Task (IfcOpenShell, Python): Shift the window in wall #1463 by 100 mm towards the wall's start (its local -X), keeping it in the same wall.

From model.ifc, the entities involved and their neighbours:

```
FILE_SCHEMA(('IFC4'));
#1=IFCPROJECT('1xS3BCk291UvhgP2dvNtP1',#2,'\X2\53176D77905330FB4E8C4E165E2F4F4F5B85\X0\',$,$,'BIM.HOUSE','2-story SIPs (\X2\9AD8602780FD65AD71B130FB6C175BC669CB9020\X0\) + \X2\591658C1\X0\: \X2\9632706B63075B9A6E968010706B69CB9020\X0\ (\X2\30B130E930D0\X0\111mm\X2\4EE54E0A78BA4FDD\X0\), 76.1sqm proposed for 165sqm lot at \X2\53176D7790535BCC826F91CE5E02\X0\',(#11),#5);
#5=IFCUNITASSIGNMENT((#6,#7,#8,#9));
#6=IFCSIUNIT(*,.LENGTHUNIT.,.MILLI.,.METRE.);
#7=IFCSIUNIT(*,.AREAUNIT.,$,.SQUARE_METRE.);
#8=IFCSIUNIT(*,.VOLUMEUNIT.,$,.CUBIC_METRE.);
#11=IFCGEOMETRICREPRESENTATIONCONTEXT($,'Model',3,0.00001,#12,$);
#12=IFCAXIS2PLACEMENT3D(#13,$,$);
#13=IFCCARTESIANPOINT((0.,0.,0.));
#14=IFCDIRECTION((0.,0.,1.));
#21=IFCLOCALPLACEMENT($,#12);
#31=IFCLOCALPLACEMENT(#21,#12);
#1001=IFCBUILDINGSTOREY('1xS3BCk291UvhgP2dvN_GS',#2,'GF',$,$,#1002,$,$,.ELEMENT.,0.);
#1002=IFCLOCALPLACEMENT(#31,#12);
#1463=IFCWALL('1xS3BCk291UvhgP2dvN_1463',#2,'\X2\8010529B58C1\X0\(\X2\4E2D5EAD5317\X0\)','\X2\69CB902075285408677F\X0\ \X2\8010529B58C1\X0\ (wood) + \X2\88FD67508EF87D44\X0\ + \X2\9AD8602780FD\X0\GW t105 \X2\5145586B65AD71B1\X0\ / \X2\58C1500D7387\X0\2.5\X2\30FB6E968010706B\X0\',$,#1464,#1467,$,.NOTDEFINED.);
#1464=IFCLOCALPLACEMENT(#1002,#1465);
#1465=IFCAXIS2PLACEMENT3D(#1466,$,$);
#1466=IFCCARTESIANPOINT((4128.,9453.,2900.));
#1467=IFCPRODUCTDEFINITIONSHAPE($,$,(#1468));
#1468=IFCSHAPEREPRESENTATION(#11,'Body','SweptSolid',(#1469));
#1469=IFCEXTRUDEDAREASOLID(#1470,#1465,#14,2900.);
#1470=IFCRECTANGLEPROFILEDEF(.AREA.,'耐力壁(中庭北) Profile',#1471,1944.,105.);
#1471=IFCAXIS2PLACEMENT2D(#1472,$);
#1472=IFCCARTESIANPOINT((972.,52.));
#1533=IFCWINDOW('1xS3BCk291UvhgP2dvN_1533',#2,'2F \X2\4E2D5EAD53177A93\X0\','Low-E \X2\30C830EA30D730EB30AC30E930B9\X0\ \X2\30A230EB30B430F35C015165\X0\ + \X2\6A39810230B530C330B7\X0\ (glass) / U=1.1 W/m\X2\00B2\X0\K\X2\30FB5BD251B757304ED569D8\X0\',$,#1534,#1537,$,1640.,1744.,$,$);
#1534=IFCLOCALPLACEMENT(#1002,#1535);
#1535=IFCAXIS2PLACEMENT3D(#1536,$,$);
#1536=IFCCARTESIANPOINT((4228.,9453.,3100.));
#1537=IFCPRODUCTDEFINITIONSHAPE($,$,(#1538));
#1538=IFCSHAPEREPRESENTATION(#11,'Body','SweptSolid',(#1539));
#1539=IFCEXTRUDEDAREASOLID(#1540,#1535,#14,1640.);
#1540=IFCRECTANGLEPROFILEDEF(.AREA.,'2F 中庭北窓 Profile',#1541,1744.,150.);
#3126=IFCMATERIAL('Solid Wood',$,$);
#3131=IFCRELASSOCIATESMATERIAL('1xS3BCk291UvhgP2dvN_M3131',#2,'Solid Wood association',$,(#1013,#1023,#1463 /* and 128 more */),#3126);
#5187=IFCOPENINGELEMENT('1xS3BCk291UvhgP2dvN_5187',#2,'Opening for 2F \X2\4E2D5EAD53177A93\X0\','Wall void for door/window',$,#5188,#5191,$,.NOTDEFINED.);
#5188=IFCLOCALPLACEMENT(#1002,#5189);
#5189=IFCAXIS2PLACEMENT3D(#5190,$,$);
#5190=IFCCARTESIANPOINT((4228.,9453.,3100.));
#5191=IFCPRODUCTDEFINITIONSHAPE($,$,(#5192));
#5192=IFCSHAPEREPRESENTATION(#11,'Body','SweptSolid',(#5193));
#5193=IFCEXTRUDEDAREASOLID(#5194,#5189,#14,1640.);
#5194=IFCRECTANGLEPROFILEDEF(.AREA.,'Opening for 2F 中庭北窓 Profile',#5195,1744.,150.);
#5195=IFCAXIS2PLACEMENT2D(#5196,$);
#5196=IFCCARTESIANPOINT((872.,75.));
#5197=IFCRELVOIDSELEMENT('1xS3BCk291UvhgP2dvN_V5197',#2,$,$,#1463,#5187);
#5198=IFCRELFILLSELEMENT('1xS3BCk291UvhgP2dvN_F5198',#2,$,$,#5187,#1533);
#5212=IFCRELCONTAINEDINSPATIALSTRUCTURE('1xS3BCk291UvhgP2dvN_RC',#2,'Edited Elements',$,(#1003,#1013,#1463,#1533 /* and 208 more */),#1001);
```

```python
import ifcopenshell
import ifcopenshell.api.geometry
import ifcopenshell.util.placement

model = ifcopenshell.open("model.ifc")

window = model.by_guid("1xS3BCk291UvhgP2dvN_1533")
opening = window.FillsVoids[0].RelatingOpeningElement
wall = opening.VoidsElements[0].RelatingBuildingElement

wall_matrix = ifcopenshell.util.placement.get_local_placement(wall.ObjectPlacement)
shift = wall_matrix[:3, 0] * -100.0
before = ifcopenshell.util.placement.get_local_placement(window.ObjectPlacement)[:3, 3].copy()

# The window is not placed relative to its opening, so move both.
for product in (opening, window):
    matrix = ifcopenshell.util.placement.get_local_placement(product.ObjectPlacement)
    matrix[:3, 3] += shift
    ifcopenshell.api.geometry.edit_object_placement(model, product=product, matrix=matrix, is_si=False)

after = ifcopenshell.util.placement.get_local_placement(window.ObjectPlacement)[:3, 3]
print("window moved by", (after - before).round(3) + 0.0)

model.write("model_rev.ifc")
```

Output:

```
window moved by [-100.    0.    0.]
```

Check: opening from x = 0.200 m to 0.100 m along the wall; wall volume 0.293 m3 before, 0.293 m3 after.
